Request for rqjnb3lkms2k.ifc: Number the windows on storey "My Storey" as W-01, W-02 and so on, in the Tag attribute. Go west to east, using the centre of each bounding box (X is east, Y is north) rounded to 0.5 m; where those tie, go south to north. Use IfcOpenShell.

First a look at what the model holds.

```python
import ifcopenshell
import ifcopenshell.util.element
import ifcopenshell.util.placement

model = ifcopenshell.open("rqjnb3lkms2k.ifc")
print(model.schema)
storey = next(s for s in model.by_type("IfcBuildingStorey") if s.Name == "My Storey")
windows = [e for e in ifcopenshell.util.element.get_decomposition(storey) if e.is_a("IfcWindow")]
for e in sorted(windows, key=lambda e: e.id()):
    origin = ifcopenshell.util.placement.get_local_placement(e.ObjectPlacement)[:3, 3]
    print(e.id(), e.Tag, e.Name, origin.round(2) + 0.0, sep=" | ")
```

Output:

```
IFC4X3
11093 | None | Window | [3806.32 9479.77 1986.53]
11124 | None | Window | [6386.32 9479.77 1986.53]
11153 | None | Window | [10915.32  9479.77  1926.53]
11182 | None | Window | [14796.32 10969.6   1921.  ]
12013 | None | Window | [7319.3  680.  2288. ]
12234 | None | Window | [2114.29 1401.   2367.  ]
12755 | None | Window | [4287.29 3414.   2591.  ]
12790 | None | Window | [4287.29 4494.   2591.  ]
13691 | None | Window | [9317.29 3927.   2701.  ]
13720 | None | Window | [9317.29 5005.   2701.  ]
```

```python
import ifcopenshell
import ifcopenshell.geom
import ifcopenshell.util.element
import ifcopenshell.util.shape

model = ifcopenshell.open("rqjnb3lkms2k.ifc")
settings = ifcopenshell.geom.settings()
settings.set("use-world-coords", True)


def centre(element):
    shape = ifcopenshell.geom.create_shape(settings, element)
    return ifcopenshell.util.shape.get_bbox_centroid(shape.geometry)


storey = next(s for s in model.by_type("IfcBuildingStorey") if s.Name == "My Storey")
windows = [e for e in ifcopenshell.util.element.get_decomposition(storey) if e.is_a("IfcWindow")]

# Insertion points can sit at a corner or the storey origin, so sort by the geometry (in metres).
centres = {e: centre(e) for e in windows}
windows.sort(key=lambda e: (round(centres[e][0] / 0.5), centres[e][1]))

for i, e in enumerate(windows, start=1):
    number = f"W-{i:02d}"
    e.Tag = number
    print(e.id(), number)

model.write("rqjnb3lkms2k-out.ifc")
```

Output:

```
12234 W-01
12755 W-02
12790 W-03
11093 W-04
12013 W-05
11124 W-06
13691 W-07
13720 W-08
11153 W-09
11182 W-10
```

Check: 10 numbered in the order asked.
